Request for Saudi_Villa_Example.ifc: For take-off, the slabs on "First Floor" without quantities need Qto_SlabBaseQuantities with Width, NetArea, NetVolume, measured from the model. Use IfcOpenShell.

First a look at what the model holds.

```python
import ifcopenshell
import ifcopenshell.util.element
import ifcopenshell.util.unit

model = ifcopenshell.open("Saudi_Villa_Example.ifc")
print(model.schema)
for unit_type in ("LENGTHUNIT", "AREAUNIT", "VOLUMEUNIT"):
    print(unit_type, ifcopenshell.util.unit.calculate_unit_scale(model, unit_type))
storey = next(s for s in model.by_type("IfcBuildingStorey") if s.Name == "First Floor")
slabs = [e for e in ifcopenshell.util.element.get_decomposition(storey) if e.is_a("IfcSlab")]
for e in sorted(slabs, key=lambda e: e.id()):
    print(e.id(), e.is_a(), e.Name, list(ifcopenshell.util.element.get_psets(e, qtos_only=True)), sep=" | ")
```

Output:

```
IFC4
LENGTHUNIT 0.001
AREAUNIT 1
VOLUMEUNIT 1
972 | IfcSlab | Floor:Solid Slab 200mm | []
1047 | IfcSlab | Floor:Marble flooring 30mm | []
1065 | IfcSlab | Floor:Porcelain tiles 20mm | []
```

```python
import ifcopenshell
import ifcopenshell.api.pset
import ifcopenshell.geom
import ifcopenshell.util.element
import ifcopenshell.util.shape
import ifcopenshell.util.unit

model = ifcopenshell.open("Saudi_Villa_Example.ifc")
unit_scale = ifcopenshell.util.unit.calculate_unit_scale(model)
area_scale = ifcopenshell.util.unit.calculate_unit_scale(model, "AREAUNIT")
volume_scale = ifcopenshell.util.unit.calculate_unit_scale(model, "VOLUMEUNIT")
settings = ifcopenshell.geom.settings()

storey = next(s for s in model.by_type("IfcBuildingStorey") if s.Name == "First Floor")
slabs = [e for e in ifcopenshell.util.element.get_decomposition(storey) if e.is_a("IfcSlab")]

for e in sorted(slabs, key=lambda e: e.id()):
    if ifcopenshell.util.element.get_psets(e, qtos_only=True, should_inherit=False):
        continue
    # Geometry comes back in metres, in the element's own axes.
    shape = ifcopenshell.geom.create_shape(settings, e)
    values = {
        "Width": ifcopenshell.util.shape.get_z(shape.geometry) / unit_scale,
        "NetArea": ifcopenshell.util.shape.get_footprint_area(shape.geometry) / area_scale,
        "NetVolume": ifcopenshell.util.shape.get_volume(shape.geometry) / volume_scale,
    }
    qto = ifcopenshell.api.pset.add_qto(model, product=e, name="Qto_SlabBaseQuantities")
    ifcopenshell.api.pset.edit_qto(model, qto=qto, properties=values)
    print(e.id(), {k: round(v, 3) for k, v in values.items()})

model.write("Saudi_Villa_Example_v2.ifc")
```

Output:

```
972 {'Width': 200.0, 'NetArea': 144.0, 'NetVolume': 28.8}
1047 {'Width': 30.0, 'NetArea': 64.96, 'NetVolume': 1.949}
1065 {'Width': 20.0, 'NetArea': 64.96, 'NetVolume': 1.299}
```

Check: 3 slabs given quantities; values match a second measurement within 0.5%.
